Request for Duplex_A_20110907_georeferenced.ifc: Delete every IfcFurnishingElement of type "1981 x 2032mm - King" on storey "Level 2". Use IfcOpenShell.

First a look at what the model holds.

```python
import ifcopenshell
import ifcopenshell.util.element

model = ifcopenshell.open("Duplex_A_20110907_georeferenced.ifc")
print(model.schema)
storey = next(s for s in model.by_type("IfcBuildingStorey") if s.Name == "Level 2")
furniture = [e for e in ifcopenshell.util.element.get_decomposition(storey) if e.is_a("IfcFurnishingElement")]
seen = {}
for e in furniture:
    element_type = ifcopenshell.util.element.get_type(e)
    name = element_type.Name if element_type not in (None, e) else None
    seen[name] = seen.get(name, 0) + 1
for name, count in sorted(seen.items(), key=str):
    print(count, "x", name)
```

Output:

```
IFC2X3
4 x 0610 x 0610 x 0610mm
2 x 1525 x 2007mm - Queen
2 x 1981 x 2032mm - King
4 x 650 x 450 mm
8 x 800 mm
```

```python
import ifcopenshell
import ifcopenshell.api.root
import ifcopenshell.util.element

model = ifcopenshell.open("Duplex_A_20110907_georeferenced.ifc")

storey = next(s for s in model.by_type("IfcBuildingStorey") if s.Name == "Level 2")
furniture = [e for e in ifcopenshell.util.element.get_decomposition(storey) if e.is_a("IfcFurnishingElement")]
targets = [e for e in furniture if (t := ifcopenshell.util.element.get_type(e)) not in (None, e) and t.Name == "1981 x 2032mm - King"]

for e in targets:
    ifcopenshell.api.root.remove_product(model, product=e)
print(len(targets), "removed")

model.write("Duplex_A_20110907_georeferenced-out.ifc")
```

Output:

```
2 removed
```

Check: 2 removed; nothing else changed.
